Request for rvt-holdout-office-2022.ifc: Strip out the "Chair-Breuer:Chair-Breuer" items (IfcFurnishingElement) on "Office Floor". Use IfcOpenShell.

First a look at what the model holds.

```python
import ifcopenshell
import ifcopenshell.util.element

model = ifcopenshell.open("rvt-holdout-office-2022.ifc")
print(model.schema)
storey = next(s for s in model.by_type("IfcBuildingStorey") if s.Name == "Office Floor")
furniture = [e for e in ifcopenshell.util.element.get_decomposition(storey) if e.is_a("IfcFurnishingElement")]
seen = {}
for e in furniture:
    element_type = ifcopenshell.util.element.get_type(e)
    name = element_type.Name if element_type not in (None, e) else None
    seen[name] = seen.get(name, 0) + 1
for name, count in sorted(seen.items(), key=str):
    print(count, "x", name)
```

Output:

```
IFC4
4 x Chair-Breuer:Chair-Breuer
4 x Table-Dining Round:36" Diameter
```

```python
import ifcopenshell
import ifcopenshell.api.root
import ifcopenshell.util.element

model = ifcopenshell.open("rvt-holdout-office-2022.ifc")

storey = next(s for s in model.by_type("IfcBuildingStorey") if s.Name == "Office Floor")
furniture = [e for e in ifcopenshell.util.element.get_decomposition(storey) if e.is_a("IfcFurnishingElement")]
targets = [e for e in furniture if (t := ifcopenshell.util.element.get_type(e)) not in (None, e) and t.Name == "Chair-Breuer:Chair-Breuer"]

for e in targets:
    ifcopenshell.api.root.remove_product(model, product=e)
print(len(targets), "removed")

model.write("rvt-holdout-office-2022_updated.ifc")
```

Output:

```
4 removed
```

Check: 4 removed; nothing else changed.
